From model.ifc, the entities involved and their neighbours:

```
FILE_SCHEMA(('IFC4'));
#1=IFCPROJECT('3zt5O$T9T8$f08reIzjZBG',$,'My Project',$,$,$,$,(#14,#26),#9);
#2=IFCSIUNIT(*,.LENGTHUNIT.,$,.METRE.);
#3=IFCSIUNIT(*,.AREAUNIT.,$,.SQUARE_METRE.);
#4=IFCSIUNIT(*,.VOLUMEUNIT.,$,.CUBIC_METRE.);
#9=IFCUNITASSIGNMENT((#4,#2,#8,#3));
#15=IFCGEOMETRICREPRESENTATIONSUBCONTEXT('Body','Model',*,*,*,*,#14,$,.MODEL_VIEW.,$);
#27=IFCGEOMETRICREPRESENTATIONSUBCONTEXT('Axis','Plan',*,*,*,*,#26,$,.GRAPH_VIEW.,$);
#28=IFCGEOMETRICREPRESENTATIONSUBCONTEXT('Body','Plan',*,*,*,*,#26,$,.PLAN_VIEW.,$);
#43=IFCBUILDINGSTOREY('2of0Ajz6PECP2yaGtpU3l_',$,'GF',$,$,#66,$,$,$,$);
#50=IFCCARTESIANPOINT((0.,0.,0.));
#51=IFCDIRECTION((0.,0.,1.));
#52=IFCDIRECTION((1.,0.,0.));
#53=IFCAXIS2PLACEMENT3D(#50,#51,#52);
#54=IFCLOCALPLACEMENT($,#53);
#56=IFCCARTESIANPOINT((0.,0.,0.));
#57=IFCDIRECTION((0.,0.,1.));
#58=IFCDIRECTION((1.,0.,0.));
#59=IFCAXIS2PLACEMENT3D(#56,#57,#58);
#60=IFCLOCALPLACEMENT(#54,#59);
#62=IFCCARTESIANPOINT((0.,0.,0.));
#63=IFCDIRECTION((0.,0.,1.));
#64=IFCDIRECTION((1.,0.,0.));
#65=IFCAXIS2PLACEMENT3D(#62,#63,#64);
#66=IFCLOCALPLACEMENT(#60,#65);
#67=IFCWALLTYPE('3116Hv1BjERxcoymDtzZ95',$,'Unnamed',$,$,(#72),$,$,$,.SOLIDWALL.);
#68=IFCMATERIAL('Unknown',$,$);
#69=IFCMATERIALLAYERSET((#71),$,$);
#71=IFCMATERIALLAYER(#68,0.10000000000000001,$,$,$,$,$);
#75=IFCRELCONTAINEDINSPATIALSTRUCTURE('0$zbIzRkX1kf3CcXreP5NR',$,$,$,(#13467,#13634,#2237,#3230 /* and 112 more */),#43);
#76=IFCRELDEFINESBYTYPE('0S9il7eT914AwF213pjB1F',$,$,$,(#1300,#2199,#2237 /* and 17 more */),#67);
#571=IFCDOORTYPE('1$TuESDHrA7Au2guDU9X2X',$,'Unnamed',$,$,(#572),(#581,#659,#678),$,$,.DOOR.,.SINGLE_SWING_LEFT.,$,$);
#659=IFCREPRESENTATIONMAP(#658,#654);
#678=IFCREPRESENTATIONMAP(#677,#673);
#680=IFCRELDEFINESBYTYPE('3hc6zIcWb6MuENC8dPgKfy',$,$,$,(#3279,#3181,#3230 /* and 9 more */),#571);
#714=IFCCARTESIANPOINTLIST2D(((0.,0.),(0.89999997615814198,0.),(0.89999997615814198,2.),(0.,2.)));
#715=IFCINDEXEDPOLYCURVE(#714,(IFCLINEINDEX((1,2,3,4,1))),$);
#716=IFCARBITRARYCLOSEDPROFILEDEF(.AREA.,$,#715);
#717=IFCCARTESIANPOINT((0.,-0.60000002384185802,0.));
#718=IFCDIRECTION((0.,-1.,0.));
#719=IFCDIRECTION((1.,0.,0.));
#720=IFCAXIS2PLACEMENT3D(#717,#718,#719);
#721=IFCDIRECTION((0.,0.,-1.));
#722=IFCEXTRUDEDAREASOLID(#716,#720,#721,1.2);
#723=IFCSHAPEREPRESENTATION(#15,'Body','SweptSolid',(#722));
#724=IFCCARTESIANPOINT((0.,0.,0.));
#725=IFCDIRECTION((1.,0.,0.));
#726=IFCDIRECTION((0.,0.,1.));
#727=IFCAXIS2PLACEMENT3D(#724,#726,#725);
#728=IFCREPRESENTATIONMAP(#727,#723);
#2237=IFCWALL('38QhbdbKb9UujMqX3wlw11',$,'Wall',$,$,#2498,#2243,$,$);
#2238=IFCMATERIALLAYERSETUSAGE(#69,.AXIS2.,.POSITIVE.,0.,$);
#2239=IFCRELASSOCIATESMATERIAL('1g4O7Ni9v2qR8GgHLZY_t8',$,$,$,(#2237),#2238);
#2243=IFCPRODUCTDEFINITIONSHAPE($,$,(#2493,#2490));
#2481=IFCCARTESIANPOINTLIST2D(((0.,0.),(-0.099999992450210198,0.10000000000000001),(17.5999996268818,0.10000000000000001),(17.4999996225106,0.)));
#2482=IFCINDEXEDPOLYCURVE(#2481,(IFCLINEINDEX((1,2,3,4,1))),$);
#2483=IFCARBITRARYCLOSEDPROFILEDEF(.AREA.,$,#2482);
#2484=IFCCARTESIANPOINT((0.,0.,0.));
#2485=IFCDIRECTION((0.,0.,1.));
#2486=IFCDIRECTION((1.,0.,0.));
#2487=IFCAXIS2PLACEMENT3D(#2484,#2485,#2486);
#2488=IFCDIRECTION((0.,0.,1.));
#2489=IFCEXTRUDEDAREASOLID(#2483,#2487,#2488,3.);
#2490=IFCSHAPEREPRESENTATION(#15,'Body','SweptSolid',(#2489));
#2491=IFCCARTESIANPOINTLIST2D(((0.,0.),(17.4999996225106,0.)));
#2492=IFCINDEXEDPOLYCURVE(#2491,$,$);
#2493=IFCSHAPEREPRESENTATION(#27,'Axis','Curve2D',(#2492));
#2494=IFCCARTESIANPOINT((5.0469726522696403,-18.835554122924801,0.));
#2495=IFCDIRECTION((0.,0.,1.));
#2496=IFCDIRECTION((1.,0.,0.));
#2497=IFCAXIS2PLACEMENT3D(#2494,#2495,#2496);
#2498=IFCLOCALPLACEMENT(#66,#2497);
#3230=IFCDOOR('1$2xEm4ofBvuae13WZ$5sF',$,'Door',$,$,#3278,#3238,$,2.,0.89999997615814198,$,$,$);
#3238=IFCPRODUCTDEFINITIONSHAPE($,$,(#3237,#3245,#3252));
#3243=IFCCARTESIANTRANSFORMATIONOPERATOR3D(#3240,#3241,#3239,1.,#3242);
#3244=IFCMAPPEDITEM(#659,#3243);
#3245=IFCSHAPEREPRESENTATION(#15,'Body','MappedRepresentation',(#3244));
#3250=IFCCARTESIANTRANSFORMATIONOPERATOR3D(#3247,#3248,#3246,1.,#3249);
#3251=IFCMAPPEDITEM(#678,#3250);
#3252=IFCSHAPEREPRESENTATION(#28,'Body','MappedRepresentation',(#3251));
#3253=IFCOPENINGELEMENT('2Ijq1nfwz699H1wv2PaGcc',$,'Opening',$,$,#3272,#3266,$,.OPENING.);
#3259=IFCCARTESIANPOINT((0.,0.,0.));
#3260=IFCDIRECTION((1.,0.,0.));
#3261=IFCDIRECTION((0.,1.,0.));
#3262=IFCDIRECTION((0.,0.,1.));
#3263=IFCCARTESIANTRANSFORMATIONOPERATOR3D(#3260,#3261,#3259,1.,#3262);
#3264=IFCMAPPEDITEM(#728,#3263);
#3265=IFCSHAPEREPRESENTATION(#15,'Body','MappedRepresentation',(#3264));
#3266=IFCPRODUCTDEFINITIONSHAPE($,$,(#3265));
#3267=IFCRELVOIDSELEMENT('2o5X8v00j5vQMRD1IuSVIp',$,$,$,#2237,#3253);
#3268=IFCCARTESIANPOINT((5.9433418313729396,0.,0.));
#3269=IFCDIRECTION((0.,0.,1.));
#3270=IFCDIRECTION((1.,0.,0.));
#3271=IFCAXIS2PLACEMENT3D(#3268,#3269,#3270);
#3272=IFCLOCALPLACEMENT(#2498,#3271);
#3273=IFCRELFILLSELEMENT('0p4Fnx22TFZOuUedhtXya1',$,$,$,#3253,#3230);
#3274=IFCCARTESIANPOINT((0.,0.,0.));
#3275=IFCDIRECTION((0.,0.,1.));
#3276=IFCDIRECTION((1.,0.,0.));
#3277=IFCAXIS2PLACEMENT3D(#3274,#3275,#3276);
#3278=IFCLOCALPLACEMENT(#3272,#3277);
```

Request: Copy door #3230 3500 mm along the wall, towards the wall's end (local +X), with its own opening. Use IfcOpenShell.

```python
import ifcopenshell
import ifcopenshell.api.feature
import ifcopenshell.api.geometry
import ifcopenshell.api.root
import ifcopenshell.geom
import ifcopenshell.util.element
import ifcopenshell.util.placement
import ifcopenshell.util.shape
import ifcopenshell.util.unit

model = ifcopenshell.open("model.ifc")
unit_scale = ifcopenshell.util.unit.calculate_unit_scale(model)
settings = ifcopenshell.geom.settings()


def volume(element):
    """Net volume in cubic metres, openings subtracted."""
    shape = ifcopenshell.geom.create_shape(settings, element)
    return ifcopenshell.util.shape.get_volume(shape.geometry)


door = model.by_guid("1$2xEm4ofBvuae13WZ$5sF")
opening = door.FillsVoids[0].RelatingOpeningElement
wall = opening.VoidsElements[0].RelatingBuildingElement
before = volume(wall)
shift = ifcopenshell.util.placement.get_local_placement(wall.ObjectPlacement)[:3, 0] * 3.5 / unit_scale

# copy_class copies the void relationship, type, container and properties, but no geometry.
new_opening = ifcopenshell.api.root.copy_class(model, product=opening)
new_opening.Representation = ifcopenshell.util.element.copy_deep(
    model, opening.Representation, exclude=["IfcGeometricRepresentationContext", "IfcRepresentationMap"]
)
new_door = ifcopenshell.api.root.copy_class(model, product=door)
new_door.Representation = ifcopenshell.util.element.copy_deep(
    model, door.Representation, exclude=["IfcGeometricRepresentationContext", "IfcRepresentationMap"]
)
ifcopenshell.api.feature.add_filling(model, opening=new_opening, element=new_door)

for old, new in ((opening, new_opening), (door, new_door)):
    matrix = ifcopenshell.util.placement.get_local_placement(old.ObjectPlacement)
    matrix[:3, 3] += shift
    ifcopenshell.api.geometry.edit_object_placement(model, product=new, matrix=matrix, is_si=False)

after = volume(wall)

print(f"wall volume {before:.3f} -> {after:.3f} m3")

model.write("model-out.ifc")
```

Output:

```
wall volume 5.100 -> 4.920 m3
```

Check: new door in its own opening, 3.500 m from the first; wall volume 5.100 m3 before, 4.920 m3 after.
